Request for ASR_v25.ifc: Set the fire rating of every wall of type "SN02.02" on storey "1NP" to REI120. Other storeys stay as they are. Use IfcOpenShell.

First a look at what the model holds.

```python
import ifcopenshell
import ifcopenshell.util.element

model = ifcopenshell.open("ASR_v25.ifc")
print(model.schema)
storey = next(s for s in model.by_type("IfcBuildingStorey") if s.Name == "1NP")
walls = [e for e in ifcopenshell.util.element.get_decomposition(storey) if e.is_a("IfcWall")]
seen = {}
for e in walls:
    element_type = ifcopenshell.util.element.get_type(e)
    key = (element_type.Name if element_type != e and element_type else None, ifcopenshell.util.element.get_pset(e, "Pset_WallCommon", "FireRating"))
    seen[key] = seen.get(key, 0) + 1
for (name, value), count in sorted(seen.items(), key=str):
    print(count, "x", name, "|", value)
```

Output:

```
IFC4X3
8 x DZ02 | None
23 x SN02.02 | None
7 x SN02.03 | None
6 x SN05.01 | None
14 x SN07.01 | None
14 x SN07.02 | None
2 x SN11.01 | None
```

```python
import ifcopenshell
import ifcopenshell.api.pset
import ifcopenshell.util.element

model = ifcopenshell.open("ASR_v25.ifc")

storey = next(s for s in model.by_type("IfcBuildingStorey") if s.Name == "1NP")
walls = [e for e in ifcopenshell.util.element.get_decomposition(storey) if e.is_a("IfcWall")]

count = 0
for e in walls:
    element_type = ifcopenshell.util.element.get_type(e)
    if element_type in (None, e) or element_type.Name != "SN02.02":
        continue
    # add_pset returns the element's existing set when there is one.
    pset = ifcopenshell.api.pset.add_pset(model, product=e, name="Pset_WallCommon")
    ifcopenshell.api.pset.edit_pset(model, pset=pset, properties={"FireRating": "REI120"})
    count += 1

print(count, "walls updated")

model.write("ASR_v25_edited.ifc")
```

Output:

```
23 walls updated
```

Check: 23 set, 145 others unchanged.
